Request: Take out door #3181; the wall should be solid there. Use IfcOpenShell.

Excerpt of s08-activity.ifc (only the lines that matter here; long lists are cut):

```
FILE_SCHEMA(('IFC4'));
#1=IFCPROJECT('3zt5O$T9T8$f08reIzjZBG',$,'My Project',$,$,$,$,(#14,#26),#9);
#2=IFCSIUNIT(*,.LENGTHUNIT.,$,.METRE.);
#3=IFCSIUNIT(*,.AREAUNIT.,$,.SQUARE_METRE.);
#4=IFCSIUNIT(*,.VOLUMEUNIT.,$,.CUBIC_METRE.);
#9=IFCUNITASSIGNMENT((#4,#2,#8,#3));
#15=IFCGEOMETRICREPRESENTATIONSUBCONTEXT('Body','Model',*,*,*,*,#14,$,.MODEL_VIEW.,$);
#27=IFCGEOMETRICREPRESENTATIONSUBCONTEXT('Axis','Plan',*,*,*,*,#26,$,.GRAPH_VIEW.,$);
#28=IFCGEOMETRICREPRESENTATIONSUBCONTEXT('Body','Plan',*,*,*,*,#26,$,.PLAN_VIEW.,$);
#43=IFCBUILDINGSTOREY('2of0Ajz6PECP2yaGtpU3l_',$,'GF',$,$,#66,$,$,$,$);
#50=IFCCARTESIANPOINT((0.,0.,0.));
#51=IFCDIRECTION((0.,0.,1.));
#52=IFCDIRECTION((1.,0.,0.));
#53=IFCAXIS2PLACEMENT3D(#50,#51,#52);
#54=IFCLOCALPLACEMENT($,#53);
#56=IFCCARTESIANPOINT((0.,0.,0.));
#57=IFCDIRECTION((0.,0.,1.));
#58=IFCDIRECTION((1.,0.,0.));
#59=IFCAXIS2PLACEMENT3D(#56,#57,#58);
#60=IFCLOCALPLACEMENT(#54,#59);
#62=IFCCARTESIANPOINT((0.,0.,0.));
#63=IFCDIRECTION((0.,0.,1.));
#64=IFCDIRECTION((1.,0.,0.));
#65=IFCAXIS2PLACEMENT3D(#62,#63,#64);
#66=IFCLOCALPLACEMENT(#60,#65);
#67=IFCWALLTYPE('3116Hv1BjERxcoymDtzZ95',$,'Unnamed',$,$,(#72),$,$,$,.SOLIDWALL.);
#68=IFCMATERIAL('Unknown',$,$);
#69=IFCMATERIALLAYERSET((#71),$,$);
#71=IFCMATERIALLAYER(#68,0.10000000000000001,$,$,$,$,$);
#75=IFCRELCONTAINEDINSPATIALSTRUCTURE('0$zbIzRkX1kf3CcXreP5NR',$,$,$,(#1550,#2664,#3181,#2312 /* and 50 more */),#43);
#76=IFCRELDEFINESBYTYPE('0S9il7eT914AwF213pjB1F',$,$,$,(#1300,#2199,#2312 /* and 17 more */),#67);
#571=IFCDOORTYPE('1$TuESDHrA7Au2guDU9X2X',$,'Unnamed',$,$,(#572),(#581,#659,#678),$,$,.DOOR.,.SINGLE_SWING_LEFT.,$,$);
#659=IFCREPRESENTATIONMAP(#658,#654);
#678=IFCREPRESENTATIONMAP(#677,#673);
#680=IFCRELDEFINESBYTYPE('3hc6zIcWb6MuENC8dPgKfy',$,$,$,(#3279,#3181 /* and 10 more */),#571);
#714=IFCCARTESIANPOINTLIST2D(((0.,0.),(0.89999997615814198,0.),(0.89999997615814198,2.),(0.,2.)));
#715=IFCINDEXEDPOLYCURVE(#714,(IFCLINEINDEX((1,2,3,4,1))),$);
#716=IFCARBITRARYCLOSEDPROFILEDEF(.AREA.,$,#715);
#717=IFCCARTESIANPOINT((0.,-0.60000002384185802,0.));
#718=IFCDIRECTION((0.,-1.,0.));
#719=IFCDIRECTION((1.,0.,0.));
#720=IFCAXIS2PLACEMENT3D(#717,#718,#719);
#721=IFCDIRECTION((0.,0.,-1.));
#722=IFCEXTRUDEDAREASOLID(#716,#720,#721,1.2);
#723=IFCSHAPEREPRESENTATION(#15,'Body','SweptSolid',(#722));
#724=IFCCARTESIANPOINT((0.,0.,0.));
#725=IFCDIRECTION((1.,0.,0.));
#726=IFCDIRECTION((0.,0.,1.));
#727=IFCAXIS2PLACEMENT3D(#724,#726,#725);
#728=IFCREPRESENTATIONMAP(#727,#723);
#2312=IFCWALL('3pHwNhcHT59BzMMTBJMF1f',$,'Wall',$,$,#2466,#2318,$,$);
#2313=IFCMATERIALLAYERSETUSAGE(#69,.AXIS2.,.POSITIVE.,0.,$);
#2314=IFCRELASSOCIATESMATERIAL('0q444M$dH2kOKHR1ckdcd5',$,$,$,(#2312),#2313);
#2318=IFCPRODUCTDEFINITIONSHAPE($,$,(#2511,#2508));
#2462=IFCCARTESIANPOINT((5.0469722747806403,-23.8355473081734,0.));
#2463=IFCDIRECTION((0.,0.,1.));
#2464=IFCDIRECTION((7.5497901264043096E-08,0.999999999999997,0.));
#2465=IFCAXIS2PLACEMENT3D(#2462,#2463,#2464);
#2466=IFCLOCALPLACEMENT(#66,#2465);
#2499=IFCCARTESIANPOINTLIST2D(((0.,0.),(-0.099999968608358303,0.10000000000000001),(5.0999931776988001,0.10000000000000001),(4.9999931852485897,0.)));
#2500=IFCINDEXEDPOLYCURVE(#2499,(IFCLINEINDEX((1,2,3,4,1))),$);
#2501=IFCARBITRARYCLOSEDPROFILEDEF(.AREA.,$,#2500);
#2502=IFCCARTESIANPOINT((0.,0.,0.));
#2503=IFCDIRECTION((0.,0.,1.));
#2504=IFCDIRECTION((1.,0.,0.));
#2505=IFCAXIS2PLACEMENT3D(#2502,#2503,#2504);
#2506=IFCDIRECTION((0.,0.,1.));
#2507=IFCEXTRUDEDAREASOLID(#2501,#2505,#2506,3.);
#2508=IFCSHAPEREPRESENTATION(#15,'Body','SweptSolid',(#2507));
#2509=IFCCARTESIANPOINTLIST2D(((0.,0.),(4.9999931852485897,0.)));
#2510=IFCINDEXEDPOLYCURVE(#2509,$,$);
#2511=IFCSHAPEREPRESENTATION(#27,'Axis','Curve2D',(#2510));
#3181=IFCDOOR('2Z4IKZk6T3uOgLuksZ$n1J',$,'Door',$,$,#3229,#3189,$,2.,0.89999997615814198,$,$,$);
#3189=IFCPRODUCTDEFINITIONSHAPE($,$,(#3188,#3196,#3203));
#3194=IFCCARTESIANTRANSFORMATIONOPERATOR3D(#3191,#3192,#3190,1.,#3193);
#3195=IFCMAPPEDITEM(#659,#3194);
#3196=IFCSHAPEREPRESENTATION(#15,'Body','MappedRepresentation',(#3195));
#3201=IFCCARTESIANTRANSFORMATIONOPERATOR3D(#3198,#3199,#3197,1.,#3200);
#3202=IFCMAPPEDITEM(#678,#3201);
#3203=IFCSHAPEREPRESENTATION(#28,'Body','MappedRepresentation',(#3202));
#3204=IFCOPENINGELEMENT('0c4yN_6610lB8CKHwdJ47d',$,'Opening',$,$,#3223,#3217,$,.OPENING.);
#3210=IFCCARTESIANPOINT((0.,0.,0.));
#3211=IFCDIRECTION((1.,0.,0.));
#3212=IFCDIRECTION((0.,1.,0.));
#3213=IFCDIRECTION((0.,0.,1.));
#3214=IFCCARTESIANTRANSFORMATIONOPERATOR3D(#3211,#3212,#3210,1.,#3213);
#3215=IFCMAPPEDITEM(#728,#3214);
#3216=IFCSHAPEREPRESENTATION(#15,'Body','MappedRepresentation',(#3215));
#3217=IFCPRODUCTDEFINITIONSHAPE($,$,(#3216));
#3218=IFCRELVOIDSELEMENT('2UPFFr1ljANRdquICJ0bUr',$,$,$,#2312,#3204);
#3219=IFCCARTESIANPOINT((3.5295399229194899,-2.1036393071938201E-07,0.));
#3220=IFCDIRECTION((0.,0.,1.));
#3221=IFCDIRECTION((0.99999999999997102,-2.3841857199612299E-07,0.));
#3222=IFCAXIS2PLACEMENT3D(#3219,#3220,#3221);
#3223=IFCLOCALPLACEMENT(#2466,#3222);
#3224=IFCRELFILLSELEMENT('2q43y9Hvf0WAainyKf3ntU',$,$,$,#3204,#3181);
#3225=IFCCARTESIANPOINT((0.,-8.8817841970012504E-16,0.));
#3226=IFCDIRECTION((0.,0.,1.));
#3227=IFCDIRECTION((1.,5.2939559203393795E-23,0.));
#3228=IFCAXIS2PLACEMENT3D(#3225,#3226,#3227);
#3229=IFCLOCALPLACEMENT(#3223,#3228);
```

```python
import ifcopenshell
import ifcopenshell.api.feature
import ifcopenshell.api.root
import ifcopenshell.geom
import ifcopenshell.util.shape

model = ifcopenshell.open("s08-activity.ifc")
settings = ifcopenshell.geom.settings()


def volume(element):
    """Net volume in cubic metres, openings subtracted."""
    shape = ifcopenshell.geom.create_shape(settings, element)
    return ifcopenshell.util.shape.get_volume(shape.geometry)


door = model.by_id(3181)
opening = door.FillsVoids[0].RelatingOpeningElement
wall = opening.VoidsElements[0].RelatingBuildingElement
before = volume(wall)

ifcopenshell.api.root.remove_product(model, product=door)
ifcopenshell.api.feature.remove_feature(model, feature=opening)

after = volume(wall)

print(f"wall volume {before:.3f} -> {after:.3f} m3")

model.write("s08-activity_rev.ifc")
```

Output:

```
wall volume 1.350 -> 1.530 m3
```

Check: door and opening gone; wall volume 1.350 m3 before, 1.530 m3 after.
